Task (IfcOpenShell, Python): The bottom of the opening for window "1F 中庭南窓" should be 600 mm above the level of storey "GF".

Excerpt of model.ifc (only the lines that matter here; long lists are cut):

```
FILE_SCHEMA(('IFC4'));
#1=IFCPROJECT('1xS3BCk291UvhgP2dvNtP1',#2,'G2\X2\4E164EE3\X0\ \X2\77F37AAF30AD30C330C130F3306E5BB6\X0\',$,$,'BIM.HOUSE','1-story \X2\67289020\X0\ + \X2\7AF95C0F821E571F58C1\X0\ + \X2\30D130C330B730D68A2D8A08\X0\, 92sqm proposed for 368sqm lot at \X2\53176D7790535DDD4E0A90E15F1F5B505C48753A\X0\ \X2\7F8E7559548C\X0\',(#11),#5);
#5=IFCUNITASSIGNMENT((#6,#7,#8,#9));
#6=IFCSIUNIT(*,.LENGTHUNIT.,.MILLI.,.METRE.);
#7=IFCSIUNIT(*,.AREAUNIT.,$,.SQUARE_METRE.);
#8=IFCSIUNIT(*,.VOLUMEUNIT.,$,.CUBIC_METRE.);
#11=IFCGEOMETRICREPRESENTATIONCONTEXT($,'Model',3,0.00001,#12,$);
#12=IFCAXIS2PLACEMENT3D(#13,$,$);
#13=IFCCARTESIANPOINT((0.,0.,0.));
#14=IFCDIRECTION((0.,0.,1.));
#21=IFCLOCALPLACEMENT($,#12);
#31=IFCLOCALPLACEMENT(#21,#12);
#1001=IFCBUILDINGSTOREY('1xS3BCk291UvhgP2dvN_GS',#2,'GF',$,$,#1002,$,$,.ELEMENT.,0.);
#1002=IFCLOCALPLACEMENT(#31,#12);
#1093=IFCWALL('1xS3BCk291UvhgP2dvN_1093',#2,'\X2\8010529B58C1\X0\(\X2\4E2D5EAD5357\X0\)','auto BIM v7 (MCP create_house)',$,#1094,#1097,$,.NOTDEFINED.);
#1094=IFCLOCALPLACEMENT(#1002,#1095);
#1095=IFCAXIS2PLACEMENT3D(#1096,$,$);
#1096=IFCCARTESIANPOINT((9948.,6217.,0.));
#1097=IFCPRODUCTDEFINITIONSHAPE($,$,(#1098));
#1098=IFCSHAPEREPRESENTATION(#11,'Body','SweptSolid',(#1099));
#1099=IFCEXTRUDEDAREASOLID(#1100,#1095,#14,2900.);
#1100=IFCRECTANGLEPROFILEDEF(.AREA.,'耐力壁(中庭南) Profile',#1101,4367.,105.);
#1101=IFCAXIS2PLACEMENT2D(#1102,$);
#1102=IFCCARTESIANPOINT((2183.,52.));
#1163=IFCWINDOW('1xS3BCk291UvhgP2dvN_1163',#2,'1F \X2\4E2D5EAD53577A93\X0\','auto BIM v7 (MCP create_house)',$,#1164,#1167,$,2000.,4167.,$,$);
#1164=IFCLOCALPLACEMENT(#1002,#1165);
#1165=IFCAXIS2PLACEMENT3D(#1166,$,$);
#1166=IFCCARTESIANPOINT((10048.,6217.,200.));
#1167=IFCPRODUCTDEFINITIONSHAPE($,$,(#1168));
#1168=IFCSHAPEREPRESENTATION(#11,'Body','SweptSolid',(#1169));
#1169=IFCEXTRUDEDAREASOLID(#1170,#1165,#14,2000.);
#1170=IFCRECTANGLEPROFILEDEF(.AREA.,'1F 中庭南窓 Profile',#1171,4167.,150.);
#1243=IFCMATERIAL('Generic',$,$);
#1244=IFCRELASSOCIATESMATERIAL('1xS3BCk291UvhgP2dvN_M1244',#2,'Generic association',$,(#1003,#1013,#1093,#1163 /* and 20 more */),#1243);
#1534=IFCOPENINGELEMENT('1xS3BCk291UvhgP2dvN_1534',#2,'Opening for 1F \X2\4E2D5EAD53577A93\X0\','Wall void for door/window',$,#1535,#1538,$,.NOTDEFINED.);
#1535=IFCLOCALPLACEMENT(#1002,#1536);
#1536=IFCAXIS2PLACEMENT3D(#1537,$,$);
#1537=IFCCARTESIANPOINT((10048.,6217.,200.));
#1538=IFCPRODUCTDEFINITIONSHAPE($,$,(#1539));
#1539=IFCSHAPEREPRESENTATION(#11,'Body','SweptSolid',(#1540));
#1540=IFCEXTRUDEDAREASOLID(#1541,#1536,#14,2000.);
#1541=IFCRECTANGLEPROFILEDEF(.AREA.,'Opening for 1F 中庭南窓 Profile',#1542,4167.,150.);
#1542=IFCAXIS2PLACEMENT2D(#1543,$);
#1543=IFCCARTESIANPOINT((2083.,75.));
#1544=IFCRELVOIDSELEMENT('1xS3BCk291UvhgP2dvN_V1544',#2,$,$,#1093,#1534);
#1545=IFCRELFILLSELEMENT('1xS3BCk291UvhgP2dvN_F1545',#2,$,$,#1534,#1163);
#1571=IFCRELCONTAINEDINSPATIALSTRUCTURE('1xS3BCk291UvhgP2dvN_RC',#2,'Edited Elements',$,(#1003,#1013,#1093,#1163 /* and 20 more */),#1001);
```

```python
import numpy as np
import ifcopenshell
import ifcopenshell.api.geometry
import ifcopenshell.geom
import ifcopenshell.util.element
import ifcopenshell.util.placement
import ifcopenshell.util.shape
import ifcopenshell.util.unit

model = ifcopenshell.open("model.ifc")
unit_scale = ifcopenshell.util.unit.calculate_unit_scale(model)

window = model.by_guid("1xS3BCk291UvhgP2dvN_1163")
opening = window.FillsVoids[0].RelatingOpeningElement
storey = ifcopenshell.util.element.get_container(window, ifc_class="IfcBuildingStorey")
level = ifcopenshell.util.placement.get_local_placement(storey.ObjectPlacement)[2, 3]

# The opening's origin need not be at the sill, so measure its lowest point.
shape = ifcopenshell.geom.create_shape(ifcopenshell.geom.settings(), opening)
bottom = ifcopenshell.util.shape.get_shape_bottom_elevation(shape, shape.geometry) / unit_scale
dz = level + 0.6 / unit_scale - bottom

shift = np.array([0.0, 0.0, dz])
# The window is not placed relative to its opening, so move both.
for product in (opening, window):
    matrix = ifcopenshell.util.placement.get_local_placement(product.ObjectPlacement)
    matrix[:3, 3] += shift
    ifcopenshell.api.geometry.edit_object_placement(model, product=product, matrix=matrix, is_si=False)

print(f"moved by {dz * unit_scale:+.3f} m")

model.write("model_updated.ifc")
```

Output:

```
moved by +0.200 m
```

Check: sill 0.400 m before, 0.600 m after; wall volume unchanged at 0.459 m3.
